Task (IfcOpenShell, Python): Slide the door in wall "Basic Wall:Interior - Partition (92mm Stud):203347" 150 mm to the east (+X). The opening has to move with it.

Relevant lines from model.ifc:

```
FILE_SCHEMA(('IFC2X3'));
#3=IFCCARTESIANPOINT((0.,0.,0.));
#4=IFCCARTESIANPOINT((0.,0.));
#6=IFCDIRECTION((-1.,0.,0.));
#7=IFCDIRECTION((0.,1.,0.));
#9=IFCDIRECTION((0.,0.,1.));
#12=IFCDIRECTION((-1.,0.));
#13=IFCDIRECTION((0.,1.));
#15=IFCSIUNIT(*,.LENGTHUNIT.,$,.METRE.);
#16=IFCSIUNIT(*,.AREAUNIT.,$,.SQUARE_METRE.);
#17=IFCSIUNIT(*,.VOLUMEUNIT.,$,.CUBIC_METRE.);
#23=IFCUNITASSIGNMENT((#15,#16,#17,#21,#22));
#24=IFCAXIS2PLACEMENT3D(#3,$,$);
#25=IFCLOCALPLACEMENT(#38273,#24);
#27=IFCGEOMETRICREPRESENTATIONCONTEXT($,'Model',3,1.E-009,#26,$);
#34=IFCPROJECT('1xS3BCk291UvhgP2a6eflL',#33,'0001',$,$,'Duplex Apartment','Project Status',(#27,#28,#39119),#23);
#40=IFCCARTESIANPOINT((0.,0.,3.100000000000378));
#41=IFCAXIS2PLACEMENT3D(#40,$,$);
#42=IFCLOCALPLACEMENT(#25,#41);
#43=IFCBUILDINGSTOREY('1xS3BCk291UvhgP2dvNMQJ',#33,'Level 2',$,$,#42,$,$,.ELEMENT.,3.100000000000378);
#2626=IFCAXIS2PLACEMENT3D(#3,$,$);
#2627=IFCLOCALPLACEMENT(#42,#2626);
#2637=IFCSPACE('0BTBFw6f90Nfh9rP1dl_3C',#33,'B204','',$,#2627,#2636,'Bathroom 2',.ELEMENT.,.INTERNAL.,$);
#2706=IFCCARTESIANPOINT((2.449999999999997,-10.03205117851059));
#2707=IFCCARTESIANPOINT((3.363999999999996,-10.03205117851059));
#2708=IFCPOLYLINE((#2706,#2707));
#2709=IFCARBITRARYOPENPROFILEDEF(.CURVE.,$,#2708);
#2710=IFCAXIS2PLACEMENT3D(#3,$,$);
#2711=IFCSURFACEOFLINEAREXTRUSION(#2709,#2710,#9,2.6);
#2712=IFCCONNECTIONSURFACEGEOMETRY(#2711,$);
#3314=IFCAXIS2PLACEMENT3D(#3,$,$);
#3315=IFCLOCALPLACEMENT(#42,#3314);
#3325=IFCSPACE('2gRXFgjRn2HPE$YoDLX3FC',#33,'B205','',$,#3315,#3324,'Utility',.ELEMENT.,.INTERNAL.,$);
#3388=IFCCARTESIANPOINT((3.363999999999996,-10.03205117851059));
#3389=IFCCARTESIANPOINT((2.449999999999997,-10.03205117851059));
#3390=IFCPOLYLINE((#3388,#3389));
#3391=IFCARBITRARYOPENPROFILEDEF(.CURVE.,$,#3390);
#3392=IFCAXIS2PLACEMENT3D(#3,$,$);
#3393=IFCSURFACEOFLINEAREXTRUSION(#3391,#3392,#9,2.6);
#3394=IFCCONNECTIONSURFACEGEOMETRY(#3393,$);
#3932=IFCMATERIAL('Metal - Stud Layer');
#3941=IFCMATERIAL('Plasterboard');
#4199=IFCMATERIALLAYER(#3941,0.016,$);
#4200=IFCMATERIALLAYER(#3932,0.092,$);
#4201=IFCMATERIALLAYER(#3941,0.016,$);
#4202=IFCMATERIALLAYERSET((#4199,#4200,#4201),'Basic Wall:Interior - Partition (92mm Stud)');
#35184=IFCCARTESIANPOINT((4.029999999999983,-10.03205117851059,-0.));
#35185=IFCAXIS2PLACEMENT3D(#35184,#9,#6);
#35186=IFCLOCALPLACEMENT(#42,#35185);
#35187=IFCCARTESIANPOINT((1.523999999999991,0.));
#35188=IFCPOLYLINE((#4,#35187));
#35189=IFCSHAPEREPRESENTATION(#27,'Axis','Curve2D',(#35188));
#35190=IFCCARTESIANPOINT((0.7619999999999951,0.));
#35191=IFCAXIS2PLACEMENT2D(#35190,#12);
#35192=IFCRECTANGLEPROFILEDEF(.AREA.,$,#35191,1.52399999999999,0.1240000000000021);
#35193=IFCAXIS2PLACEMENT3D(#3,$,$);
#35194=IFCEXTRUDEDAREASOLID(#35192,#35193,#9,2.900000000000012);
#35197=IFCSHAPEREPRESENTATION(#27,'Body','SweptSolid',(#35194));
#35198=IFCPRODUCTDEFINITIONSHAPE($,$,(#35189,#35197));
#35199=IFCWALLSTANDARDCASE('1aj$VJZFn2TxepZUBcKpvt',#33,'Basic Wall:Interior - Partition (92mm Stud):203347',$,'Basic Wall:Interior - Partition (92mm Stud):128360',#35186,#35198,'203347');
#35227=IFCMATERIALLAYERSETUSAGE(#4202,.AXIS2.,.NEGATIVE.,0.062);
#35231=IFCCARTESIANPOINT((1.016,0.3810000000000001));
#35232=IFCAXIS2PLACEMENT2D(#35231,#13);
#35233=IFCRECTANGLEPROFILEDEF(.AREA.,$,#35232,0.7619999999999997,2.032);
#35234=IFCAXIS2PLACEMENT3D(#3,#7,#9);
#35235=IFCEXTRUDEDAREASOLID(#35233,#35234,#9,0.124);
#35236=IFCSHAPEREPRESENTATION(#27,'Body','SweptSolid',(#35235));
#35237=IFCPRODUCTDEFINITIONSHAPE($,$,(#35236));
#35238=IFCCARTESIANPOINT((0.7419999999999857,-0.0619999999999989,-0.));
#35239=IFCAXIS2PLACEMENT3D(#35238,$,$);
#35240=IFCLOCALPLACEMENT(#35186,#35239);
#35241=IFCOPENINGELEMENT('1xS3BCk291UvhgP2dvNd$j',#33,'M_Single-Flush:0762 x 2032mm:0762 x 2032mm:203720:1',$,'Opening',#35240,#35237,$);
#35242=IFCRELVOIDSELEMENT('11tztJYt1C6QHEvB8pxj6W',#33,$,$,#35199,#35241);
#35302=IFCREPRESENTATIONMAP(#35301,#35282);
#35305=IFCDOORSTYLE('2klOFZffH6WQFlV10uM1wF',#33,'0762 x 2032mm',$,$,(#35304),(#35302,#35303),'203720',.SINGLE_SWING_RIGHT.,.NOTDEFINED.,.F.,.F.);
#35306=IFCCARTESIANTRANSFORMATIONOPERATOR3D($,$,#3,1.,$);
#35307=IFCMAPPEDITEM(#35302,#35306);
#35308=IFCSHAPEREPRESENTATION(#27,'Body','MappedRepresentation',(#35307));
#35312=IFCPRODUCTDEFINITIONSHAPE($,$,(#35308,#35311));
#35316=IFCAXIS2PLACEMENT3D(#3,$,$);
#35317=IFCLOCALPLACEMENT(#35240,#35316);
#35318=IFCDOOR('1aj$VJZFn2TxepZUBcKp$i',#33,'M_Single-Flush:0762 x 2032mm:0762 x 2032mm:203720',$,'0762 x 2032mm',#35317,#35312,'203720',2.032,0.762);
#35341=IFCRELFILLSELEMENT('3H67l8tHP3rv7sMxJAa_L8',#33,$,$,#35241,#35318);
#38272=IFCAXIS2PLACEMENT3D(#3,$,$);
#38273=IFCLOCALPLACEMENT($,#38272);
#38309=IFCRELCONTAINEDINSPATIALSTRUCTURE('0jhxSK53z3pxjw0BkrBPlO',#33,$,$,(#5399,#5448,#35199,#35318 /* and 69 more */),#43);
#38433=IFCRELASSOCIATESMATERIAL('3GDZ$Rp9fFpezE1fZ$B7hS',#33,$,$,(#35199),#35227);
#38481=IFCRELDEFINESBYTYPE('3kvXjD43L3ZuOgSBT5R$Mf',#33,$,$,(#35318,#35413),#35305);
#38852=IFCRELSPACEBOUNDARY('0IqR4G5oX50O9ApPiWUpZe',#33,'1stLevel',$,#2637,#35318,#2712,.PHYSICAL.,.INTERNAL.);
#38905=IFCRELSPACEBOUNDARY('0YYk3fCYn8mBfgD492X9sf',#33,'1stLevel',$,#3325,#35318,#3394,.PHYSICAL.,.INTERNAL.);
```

```python
import numpy as np
import ifcopenshell
import ifcopenshell.api.geometry
import ifcopenshell.util.placement
import ifcopenshell.util.unit

model = ifcopenshell.open("model.ifc")
unit_scale = ifcopenshell.util.unit.calculate_unit_scale(model)

door = model.by_guid("1aj$VJZFn2TxepZUBcKp$i")
opening = door.FillsVoids[0].RelatingOpeningElement
wall = opening.VoidsElements[0].RelatingBuildingElement

wall_matrix = ifcopenshell.util.placement.get_local_placement(wall.ObjectPlacement)
shift = wall_matrix[:3, 0] * -0.15 / unit_scale
before = ifcopenshell.util.placement.get_local_placement(door.ObjectPlacement)[:3, 3].copy()

# The door is placed relative to its opening, so it follows when the opening moves.
matrix = ifcopenshell.util.placement.get_local_placement(opening.ObjectPlacement)
matrix[:3, 3] += shift
ifcopenshell.api.geometry.edit_object_placement(
    model, product=opening, matrix=matrix, is_si=False, should_transform_children=True
)

# Space boundary surfaces are stored in each space's coordinates; move them too.
for rel in door.ProvidesBoundaries:
    if not rel.ConnectionGeometry:
        continue
    surface = rel.ConnectionGeometry.SurfaceOnRelatingElement
    space_matrix = ifcopenshell.util.placement.get_local_placement(rel.RelatingSpace.ObjectPlacement)
    point = np.array(surface.Position.Location.Coordinates) + space_matrix[:3, :3].T @ shift
    surface.Position = model.createIfcAxis2Placement3D(
        model.createIfcCartesianPoint(point.tolist()), surface.Position.Axis, surface.Position.RefDirection
    )

after = ifcopenshell.util.placement.get_local_placement(door.ObjectPlacement)[:3, 3]
print("door moved by", (after - before).round(3) + 0.0)

model.write("model_rev.ifc")
```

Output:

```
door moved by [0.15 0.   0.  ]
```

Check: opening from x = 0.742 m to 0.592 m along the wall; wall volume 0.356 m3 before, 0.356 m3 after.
